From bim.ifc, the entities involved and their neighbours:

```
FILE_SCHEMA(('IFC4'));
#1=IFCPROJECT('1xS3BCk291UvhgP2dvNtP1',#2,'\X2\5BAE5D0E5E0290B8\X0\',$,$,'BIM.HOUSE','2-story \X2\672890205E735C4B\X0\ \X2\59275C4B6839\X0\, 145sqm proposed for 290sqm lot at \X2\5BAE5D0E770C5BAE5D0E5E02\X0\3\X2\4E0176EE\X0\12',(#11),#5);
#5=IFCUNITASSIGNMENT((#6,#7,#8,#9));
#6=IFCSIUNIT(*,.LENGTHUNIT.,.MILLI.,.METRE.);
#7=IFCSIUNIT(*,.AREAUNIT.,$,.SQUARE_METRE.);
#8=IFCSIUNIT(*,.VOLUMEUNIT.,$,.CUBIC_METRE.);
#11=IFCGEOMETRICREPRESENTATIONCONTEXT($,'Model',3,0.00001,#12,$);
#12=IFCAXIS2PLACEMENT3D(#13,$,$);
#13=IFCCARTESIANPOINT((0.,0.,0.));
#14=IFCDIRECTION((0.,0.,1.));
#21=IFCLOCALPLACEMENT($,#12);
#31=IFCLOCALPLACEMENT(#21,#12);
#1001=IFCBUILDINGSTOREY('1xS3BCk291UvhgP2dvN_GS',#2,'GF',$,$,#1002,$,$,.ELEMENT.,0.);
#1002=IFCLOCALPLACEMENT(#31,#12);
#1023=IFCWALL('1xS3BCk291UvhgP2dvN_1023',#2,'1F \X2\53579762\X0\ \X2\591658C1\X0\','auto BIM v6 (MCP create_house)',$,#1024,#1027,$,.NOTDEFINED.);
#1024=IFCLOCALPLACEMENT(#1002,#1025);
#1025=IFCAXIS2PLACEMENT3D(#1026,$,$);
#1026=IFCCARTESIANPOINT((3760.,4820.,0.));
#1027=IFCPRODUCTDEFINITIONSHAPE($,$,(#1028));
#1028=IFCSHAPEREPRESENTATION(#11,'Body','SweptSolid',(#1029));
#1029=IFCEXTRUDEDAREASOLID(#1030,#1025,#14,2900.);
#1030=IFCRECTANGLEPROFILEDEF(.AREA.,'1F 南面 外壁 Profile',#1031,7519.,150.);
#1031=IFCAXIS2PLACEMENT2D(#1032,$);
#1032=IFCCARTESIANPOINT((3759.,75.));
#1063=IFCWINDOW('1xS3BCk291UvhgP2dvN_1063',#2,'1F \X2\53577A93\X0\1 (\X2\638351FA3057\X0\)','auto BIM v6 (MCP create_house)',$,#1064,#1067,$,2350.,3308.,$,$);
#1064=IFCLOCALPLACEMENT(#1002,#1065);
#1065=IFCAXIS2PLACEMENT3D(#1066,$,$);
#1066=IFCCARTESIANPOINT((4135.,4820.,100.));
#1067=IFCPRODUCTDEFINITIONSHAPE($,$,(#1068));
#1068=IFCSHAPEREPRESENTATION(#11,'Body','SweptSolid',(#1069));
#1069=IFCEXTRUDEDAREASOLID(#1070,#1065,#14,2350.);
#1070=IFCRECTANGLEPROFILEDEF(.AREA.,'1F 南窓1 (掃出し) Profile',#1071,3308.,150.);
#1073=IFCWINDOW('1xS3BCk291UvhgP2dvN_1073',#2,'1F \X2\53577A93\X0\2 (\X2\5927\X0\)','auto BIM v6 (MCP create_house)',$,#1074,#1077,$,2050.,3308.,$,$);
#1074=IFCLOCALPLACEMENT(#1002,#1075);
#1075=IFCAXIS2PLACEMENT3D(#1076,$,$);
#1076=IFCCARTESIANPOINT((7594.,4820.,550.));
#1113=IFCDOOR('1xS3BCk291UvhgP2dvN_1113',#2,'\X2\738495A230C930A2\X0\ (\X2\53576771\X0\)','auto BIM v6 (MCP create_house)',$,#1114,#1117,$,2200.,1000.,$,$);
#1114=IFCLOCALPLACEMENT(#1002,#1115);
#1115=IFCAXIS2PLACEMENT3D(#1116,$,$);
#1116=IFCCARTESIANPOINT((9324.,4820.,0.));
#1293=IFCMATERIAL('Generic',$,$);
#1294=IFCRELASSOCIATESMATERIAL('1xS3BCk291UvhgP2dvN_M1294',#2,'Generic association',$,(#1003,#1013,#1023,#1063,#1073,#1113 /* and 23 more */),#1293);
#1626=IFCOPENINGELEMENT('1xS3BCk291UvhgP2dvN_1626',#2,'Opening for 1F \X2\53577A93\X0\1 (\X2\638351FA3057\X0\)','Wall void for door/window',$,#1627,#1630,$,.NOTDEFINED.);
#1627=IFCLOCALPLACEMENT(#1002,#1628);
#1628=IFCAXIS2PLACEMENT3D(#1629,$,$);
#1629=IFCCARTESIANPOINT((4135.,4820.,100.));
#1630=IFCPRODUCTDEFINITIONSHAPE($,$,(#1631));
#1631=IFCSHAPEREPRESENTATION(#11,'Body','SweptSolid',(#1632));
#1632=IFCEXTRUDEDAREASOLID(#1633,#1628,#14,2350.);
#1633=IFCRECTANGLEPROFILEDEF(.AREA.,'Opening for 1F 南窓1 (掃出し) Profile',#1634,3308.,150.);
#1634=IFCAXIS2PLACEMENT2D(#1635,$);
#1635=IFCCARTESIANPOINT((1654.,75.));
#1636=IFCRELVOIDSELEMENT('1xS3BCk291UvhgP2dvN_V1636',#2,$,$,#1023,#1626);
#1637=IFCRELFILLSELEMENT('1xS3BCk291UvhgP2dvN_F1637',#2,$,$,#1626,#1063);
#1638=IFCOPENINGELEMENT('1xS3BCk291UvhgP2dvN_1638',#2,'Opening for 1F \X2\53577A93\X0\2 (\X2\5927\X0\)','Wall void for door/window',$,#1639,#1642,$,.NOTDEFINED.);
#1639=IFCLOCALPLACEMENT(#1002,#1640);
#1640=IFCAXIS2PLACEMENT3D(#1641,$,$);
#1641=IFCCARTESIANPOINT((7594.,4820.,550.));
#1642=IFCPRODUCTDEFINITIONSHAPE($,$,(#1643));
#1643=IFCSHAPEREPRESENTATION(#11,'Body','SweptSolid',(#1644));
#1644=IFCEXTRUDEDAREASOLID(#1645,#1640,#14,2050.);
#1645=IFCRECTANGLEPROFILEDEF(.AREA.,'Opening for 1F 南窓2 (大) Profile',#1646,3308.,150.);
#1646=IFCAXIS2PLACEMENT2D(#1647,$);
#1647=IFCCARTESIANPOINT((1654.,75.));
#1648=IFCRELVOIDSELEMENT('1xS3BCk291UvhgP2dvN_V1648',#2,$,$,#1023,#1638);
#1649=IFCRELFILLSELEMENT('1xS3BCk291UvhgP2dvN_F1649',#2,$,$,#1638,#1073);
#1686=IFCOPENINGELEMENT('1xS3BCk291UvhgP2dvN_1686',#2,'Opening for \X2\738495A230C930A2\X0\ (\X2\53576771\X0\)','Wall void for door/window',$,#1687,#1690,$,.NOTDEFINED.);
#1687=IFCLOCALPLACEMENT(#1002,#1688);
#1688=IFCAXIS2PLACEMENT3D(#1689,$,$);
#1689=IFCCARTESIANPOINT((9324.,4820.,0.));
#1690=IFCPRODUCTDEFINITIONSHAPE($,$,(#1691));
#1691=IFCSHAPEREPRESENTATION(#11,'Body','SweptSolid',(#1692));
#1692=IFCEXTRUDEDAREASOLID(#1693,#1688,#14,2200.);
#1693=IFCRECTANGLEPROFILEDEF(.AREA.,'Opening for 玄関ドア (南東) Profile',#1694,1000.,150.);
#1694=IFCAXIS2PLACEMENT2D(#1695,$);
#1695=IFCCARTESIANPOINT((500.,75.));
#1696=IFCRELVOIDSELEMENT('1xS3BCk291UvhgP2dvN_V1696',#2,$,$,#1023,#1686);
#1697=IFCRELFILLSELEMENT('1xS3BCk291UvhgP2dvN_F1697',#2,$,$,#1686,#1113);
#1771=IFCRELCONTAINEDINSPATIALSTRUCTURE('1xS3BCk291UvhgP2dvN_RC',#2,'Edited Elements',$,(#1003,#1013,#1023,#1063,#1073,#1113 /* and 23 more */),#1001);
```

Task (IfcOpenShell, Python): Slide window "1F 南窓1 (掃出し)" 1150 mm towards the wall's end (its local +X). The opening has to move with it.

```python
import ifcopenshell
import ifcopenshell.api.geometry
import ifcopenshell.util.placement
import ifcopenshell.util.unit

model = ifcopenshell.open("bim.ifc")
unit_scale = ifcopenshell.util.unit.calculate_unit_scale(model)

window = model.by_id(1063)
opening = window.FillsVoids[0].RelatingOpeningElement
wall = opening.VoidsElements[0].RelatingBuildingElement

wall_matrix = ifcopenshell.util.placement.get_local_placement(wall.ObjectPlacement)
shift = wall_matrix[:3, 0] * 1.15 / unit_scale
before = ifcopenshell.util.placement.get_local_placement(window.ObjectPlacement)[:3, 3].copy()

# The window is not placed relative to its opening, so move both.
for product in (opening, window):
    matrix = ifcopenshell.util.placement.get_local_placement(product.ObjectPlacement)
    matrix[:3, 3] += shift
    ifcopenshell.api.geometry.edit_object_placement(model, product=product, matrix=matrix, is_si=False)

after = ifcopenshell.util.placement.get_local_placement(window.ObjectPlacement)[:3, 3]
print("window moved by", (after - before).round(3) + 0.0)

model.write("bim_updated.ifc")
```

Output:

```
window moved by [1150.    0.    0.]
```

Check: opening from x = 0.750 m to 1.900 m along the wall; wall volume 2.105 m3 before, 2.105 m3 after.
